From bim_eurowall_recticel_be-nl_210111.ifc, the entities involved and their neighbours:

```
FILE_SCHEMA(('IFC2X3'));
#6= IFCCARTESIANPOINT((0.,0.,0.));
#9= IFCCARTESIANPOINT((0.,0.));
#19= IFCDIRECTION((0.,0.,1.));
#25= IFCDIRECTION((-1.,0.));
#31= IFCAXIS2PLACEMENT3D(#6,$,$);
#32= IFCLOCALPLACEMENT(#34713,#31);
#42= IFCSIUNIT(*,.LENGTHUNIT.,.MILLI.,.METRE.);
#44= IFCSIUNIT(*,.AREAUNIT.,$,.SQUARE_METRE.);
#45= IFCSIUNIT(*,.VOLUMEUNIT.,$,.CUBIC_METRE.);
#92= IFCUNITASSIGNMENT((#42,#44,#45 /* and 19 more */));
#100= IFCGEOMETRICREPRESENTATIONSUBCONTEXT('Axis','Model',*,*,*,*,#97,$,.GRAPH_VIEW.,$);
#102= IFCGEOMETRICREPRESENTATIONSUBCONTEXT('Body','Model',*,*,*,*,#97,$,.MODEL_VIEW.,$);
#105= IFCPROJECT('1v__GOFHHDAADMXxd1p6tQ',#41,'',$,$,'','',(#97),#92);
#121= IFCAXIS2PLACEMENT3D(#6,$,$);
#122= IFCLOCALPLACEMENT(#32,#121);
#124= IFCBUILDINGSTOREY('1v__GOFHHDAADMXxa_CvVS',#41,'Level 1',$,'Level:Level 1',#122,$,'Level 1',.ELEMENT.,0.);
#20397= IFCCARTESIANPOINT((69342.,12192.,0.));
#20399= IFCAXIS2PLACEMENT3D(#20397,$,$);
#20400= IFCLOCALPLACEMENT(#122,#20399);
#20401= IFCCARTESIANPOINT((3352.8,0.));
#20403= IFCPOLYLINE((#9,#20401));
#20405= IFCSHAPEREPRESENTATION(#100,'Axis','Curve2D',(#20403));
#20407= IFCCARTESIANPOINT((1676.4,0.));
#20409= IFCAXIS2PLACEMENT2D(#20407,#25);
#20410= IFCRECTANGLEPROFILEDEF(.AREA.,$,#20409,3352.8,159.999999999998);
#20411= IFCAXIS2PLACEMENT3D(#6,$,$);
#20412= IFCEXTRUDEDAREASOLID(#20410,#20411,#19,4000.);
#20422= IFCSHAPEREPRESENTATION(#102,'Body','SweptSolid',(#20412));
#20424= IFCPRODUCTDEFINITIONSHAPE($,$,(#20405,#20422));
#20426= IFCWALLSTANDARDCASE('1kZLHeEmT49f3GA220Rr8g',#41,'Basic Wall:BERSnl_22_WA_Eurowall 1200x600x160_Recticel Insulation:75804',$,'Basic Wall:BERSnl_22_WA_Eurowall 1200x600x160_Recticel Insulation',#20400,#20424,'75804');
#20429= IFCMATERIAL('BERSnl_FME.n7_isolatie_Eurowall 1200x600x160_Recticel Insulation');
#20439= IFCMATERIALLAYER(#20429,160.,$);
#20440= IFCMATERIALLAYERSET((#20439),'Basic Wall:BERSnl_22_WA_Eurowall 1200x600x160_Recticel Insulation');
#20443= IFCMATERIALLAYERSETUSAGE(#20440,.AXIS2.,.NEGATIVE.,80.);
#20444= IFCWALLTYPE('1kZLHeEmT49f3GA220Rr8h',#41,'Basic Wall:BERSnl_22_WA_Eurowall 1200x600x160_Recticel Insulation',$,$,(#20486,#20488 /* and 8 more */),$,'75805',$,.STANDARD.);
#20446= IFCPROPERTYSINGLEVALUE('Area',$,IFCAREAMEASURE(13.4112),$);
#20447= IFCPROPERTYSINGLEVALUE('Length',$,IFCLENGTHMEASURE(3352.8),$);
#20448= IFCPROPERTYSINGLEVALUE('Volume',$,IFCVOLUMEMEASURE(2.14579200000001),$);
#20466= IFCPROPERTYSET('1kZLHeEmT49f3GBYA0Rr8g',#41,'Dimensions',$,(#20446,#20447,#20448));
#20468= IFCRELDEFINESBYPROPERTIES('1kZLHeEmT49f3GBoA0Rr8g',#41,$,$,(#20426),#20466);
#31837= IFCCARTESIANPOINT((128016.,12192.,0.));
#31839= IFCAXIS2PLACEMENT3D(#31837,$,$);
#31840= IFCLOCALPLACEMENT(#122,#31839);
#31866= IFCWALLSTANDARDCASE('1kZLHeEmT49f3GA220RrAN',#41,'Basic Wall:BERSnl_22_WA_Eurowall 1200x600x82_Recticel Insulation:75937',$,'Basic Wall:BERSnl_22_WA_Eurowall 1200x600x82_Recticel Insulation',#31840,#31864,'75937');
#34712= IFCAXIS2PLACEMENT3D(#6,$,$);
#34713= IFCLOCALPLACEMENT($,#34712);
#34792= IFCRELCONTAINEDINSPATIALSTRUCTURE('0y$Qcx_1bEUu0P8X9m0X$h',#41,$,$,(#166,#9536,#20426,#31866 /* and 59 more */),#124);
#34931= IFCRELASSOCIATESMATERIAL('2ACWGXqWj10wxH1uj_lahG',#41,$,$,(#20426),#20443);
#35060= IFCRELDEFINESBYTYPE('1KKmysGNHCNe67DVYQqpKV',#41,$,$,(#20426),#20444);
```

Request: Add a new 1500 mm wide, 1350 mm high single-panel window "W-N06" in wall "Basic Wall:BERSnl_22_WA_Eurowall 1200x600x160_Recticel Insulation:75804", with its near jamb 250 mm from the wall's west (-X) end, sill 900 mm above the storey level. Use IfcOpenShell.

```python
import numpy as np
import ifcopenshell
import ifcopenshell.api.feature
import ifcopenshell.api.geometry
import ifcopenshell.api.pset
import ifcopenshell.api.root
import ifcopenshell.api.spatial
import ifcopenshell.api.type
import ifcopenshell.geom
import ifcopenshell.util.element
import ifcopenshell.util.placement
import ifcopenshell.util.representation
import ifcopenshell.util.shape
import ifcopenshell.util.unit

model = ifcopenshell.open("bim_eurowall_recticel_be-nl_210111.ifc")
unit_scale = ifcopenshell.util.unit.calculate_unit_scale(model)
area_scale = ifcopenshell.util.unit.calculate_unit_scale(model, "AREAUNIT")
volume_scale = ifcopenshell.util.unit.calculate_unit_scale(model, "VOLUMEUNIT")
settings = ifcopenshell.geom.settings()


def volume(element):
    """Net volume in cubic metres, openings subtracted."""
    shape = ifcopenshell.geom.create_shape(settings, element)
    return ifcopenshell.util.shape.get_volume(shape.geometry)


wall = model.by_guid("1kZLHeEmT49f3GA220Rr8g")
storey = ifcopenshell.util.element.get_container(wall, ifc_class="IfcBuildingStorey")
context = ifcopenshell.util.representation.get_context(model, "Model", "Body", "MODEL_VIEW")
before = volume(wall)

width, height, from_end, sill = 1.5, 1.35, 0.25, 0.9  # metres

# The wall runs along its own X axis, and the end named is its -X end.
wall_shape = ifcopenshell.geom.create_shape(settings, wall)
x, y, z = ifcopenshell.util.shape.get_vertices(wall_shape.geometry).T
start = x.min() + from_end
face, thickness = float(y.min()), float(y.max() - y.min())
wall_matrix = ifcopenshell.util.placement.get_local_placement(wall.ObjectPlacement)
level = ifcopenshell.util.placement.get_local_placement(storey.ObjectPlacement)[2, 3]


def in_wall(x, y):
    """Placement at x, y metres in the wall's axes, at sill height."""
    matrix = wall_matrix.copy()
    matrix[:, 3] = wall_matrix @ np.array([x / unit_scale, y / unit_scale, 0.0, 1.0])
    matrix[2, 3] = level + sill / unit_scale
    return matrix


# Opening: a box that overshoots both wall faces by 50 mm.
opening = ifcopenshell.api.root.create_entity(model, ifc_class="IfcOpeningElement")
box = ifcopenshell.api.geometry.add_wall_representation(
    model, context=context, length=width, height=height, thickness=thickness + 0.1
)
ifcopenshell.api.geometry.assign_representation(model, product=opening, representation=box)
ifcopenshell.api.geometry.edit_object_placement(model, product=opening, matrix=in_wall(start, face - 0.05), is_si=False)
ifcopenshell.api.feature.add_feature(model, feature=opening, element=wall)

window = ifcopenshell.api.root.create_entity(model, ifc_class="IfcWindow", name="W-N06")
window.OverallWidth, window.OverallHeight = width / unit_scale, height / unit_scale
body = ifcopenshell.api.geometry.add_window_representation(
    model,
    context=context,
    overall_width=window.OverallWidth,
    overall_height=window.OverallHeight,
    partition_type="SINGLE_PANEL",
)
ifcopenshell.api.geometry.assign_representation(model, product=window, representation=body)
ifcopenshell.api.spatial.assign_container(model, products=[window], relating_structure=storey)
fills = ifcopenshell.api.feature.add_filling(model, opening=opening, element=window)
fills.OwnerHistory = window.OwnerHistory  # required in IFC2X3

# IFC2X3 keeps the operation on the window style.
style = ifcopenshell.api.root.create_entity(model, ifc_class="IfcWindowStyle", name="W-N06")
style.OperationType, style.ConstructionType = "SINGLE_PANEL", "NOTDEFINED"
style.ParameterTakesPrecedence = style.Sizeable = False
ifcopenshell.api.type.assign_type(model, related_objects=[window], relating_type=style)

# Centre the window in the wall's thickness.
ifcopenshell.api.geometry.edit_object_placement(model, product=window, matrix=in_wall(start, face), is_si=False)
window_shape = ifcopenshell.geom.create_shape(settings, window)
depth = ifcopenshell.util.shape.get_vertices(window_shape.geometry)[:, 1]
offset = face + thickness / 2 - (depth.min() + depth.max()) / 2
ifcopenshell.api.geometry.edit_object_placement(model, product=window, matrix=in_wall(start, offset), is_si=False)

after = volume(wall)

# Update the wall's stored quantities.
pset = model.by_id(ifcopenshell.util.element.get_pset(wall, "Dimensions", should_inherit=False)["id"])
ifcopenshell.api.pset.edit_pset(model, pset=pset, properties={
    "Area": model.create_entity("IfcAreaMeasure", after / thickness / area_scale),
    "Volume": model.create_entity("IfcVolumeMeasure", after / volume_scale),
})

print(f"wall volume {before:.3f} -> {after:.3f} m3")

model.write("bim_eurowall_recticel_be-nl_210111-out.ifc")
```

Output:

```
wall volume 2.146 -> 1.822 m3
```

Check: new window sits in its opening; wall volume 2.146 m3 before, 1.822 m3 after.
